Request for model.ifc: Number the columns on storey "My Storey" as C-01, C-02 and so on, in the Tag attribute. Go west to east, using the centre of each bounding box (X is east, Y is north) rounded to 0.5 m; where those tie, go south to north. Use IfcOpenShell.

First a look at what the model holds.

```python
import ifcopenshell
import ifcopenshell.util.element
import ifcopenshell.util.placement

model = ifcopenshell.open("model.ifc")
print(model.schema)
storey = next(s for s in model.by_type("IfcBuildingStorey") if s.Name == "My Storey")
columns = [e for e in ifcopenshell.util.element.get_decomposition(storey) if e.is_a("IfcColumn")]
for e in sorted(columns, key=lambda e: e.id()):
    origin = ifcopenshell.util.placement.get_local_placement(e.ObjectPlacement)[:3, 3]
    print(e.id(), e.Tag, e.Name, origin.round(2) + 0.0, sep=" | ")
```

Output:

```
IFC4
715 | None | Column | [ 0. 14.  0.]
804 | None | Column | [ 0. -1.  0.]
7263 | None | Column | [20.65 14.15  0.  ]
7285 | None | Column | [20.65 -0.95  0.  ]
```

```python
import ifcopenshell
import ifcopenshell.geom
import ifcopenshell.util.element
import ifcopenshell.util.shape

model = ifcopenshell.open("model.ifc")
settings = ifcopenshell.geom.settings()
settings.set("use-world-coords", True)


def centre(element):
    shape = ifcopenshell.geom.create_shape(settings, element)
    return ifcopenshell.util.shape.get_bbox_centroid(shape.geometry)


storey = next(s for s in model.by_type("IfcBuildingStorey") if s.Name == "My Storey")
columns = [e for e in ifcopenshell.util.element.get_decomposition(storey) if e.is_a("IfcColumn")]

# Insertion points can sit at a corner or the storey origin, so sort by the geometry (in metres).
centres = {e: centre(e) for e in columns}
columns.sort(key=lambda e: (round(centres[e][0] / 0.5), centres[e][1]))

for i, e in enumerate(columns, start=1):
    number = f"C-{i:02d}"
    e.Tag = number
    print(e.id(), number)

model.write("model_rev.ifc")
```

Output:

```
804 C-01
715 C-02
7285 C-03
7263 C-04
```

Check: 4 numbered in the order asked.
